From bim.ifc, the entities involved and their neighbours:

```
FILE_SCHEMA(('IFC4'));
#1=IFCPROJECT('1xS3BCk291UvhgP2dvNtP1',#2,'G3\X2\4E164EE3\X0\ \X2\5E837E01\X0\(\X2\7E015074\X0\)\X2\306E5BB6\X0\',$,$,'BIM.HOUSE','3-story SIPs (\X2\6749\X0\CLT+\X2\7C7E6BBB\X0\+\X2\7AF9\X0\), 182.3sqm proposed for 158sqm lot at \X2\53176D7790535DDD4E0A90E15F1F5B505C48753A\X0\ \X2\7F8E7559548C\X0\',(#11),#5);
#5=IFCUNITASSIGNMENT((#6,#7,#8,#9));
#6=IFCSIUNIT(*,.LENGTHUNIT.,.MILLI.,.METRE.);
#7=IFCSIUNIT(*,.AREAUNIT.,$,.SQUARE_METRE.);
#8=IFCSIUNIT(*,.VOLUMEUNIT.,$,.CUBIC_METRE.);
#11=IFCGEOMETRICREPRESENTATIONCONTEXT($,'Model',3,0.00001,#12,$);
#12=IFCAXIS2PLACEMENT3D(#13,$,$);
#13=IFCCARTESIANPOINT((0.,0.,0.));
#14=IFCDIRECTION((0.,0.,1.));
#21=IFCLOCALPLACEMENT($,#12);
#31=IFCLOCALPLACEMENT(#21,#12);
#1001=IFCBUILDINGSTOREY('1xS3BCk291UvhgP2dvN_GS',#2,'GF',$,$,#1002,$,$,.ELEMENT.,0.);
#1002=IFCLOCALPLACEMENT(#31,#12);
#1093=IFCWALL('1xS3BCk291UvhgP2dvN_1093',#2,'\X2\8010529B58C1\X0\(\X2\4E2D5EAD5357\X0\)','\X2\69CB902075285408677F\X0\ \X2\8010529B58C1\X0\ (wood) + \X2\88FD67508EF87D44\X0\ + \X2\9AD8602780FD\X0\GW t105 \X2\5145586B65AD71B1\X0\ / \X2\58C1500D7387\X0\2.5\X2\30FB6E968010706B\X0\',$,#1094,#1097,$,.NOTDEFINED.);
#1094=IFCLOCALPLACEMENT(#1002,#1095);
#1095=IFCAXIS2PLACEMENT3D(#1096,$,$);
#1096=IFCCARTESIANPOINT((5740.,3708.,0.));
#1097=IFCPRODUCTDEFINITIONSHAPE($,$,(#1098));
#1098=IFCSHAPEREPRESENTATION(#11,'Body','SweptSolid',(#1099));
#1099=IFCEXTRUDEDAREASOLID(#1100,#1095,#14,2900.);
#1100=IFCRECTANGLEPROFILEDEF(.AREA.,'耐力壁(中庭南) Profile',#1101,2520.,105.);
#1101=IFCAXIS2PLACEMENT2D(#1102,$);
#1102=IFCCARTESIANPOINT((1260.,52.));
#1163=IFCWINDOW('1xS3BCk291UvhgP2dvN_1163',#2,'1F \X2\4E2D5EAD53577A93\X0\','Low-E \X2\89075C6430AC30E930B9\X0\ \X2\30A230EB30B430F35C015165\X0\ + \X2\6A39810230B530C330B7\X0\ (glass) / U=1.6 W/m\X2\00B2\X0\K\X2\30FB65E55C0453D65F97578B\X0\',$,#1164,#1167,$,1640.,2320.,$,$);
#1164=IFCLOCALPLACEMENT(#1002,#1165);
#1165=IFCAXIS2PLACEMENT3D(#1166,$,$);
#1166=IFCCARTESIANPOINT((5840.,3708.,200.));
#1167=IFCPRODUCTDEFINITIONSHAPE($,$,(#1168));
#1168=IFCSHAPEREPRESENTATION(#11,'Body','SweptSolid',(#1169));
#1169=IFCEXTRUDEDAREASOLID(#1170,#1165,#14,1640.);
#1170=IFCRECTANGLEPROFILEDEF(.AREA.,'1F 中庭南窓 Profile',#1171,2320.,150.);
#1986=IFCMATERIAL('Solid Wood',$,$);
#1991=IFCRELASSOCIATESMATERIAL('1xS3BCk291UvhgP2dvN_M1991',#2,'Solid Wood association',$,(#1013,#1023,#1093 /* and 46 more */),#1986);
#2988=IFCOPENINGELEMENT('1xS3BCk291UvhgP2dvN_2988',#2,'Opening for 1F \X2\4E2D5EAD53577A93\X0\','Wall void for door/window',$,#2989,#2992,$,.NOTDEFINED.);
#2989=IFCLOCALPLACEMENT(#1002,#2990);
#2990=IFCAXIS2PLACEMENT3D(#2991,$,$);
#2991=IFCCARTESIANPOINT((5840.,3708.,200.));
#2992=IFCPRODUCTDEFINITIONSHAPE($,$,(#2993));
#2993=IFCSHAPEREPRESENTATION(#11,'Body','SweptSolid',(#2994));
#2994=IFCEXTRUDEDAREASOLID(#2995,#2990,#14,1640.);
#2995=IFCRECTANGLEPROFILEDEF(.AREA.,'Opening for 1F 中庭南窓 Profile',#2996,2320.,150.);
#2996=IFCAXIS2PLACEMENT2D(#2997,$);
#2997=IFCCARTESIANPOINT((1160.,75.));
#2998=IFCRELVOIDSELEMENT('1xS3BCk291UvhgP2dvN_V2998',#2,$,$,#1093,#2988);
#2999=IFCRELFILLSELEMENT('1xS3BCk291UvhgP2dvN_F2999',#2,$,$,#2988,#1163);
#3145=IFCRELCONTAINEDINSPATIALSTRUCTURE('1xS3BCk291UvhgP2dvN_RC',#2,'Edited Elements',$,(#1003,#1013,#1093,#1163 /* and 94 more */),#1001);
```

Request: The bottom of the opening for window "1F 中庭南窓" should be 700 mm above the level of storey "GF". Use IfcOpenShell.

```python
import numpy as np
import ifcopenshell
import ifcopenshell.api.geometry
import ifcopenshell.geom
import ifcopenshell.util.element
import ifcopenshell.util.placement
import ifcopenshell.util.shape
import ifcopenshell.util.unit

model = ifcopenshell.open("bim.ifc")
unit_scale = ifcopenshell.util.unit.calculate_unit_scale(model)

window = model.by_guid("1xS3BCk291UvhgP2dvN_1163")
opening = window.FillsVoids[0].RelatingOpeningElement
storey = ifcopenshell.util.element.get_container(window, ifc_class="IfcBuildingStorey")
level = ifcopenshell.util.placement.get_local_placement(storey.ObjectPlacement)[2, 3]

# The opening's origin need not be at the sill, so measure its lowest point.
shape = ifcopenshell.geom.create_shape(ifcopenshell.geom.settings(), opening)
bottom = ifcopenshell.util.shape.get_shape_bottom_elevation(shape, shape.geometry) / unit_scale
dz = level + 700.0 - bottom

shift = np.array([0.0, 0.0, dz])
# The window is not placed relative to its opening, so move both.
for product in (opening, window):
    matrix = ifcopenshell.util.placement.get_local_placement(product.ObjectPlacement)
    matrix[:3, 3] += shift
    ifcopenshell.api.geometry.edit_object_placement(model, product=product, matrix=matrix, is_si=False)

print(f"moved by {dz * unit_scale:+.3f} m")

model.write("bim_v2.ifc")
```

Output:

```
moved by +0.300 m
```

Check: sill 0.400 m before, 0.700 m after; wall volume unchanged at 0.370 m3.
